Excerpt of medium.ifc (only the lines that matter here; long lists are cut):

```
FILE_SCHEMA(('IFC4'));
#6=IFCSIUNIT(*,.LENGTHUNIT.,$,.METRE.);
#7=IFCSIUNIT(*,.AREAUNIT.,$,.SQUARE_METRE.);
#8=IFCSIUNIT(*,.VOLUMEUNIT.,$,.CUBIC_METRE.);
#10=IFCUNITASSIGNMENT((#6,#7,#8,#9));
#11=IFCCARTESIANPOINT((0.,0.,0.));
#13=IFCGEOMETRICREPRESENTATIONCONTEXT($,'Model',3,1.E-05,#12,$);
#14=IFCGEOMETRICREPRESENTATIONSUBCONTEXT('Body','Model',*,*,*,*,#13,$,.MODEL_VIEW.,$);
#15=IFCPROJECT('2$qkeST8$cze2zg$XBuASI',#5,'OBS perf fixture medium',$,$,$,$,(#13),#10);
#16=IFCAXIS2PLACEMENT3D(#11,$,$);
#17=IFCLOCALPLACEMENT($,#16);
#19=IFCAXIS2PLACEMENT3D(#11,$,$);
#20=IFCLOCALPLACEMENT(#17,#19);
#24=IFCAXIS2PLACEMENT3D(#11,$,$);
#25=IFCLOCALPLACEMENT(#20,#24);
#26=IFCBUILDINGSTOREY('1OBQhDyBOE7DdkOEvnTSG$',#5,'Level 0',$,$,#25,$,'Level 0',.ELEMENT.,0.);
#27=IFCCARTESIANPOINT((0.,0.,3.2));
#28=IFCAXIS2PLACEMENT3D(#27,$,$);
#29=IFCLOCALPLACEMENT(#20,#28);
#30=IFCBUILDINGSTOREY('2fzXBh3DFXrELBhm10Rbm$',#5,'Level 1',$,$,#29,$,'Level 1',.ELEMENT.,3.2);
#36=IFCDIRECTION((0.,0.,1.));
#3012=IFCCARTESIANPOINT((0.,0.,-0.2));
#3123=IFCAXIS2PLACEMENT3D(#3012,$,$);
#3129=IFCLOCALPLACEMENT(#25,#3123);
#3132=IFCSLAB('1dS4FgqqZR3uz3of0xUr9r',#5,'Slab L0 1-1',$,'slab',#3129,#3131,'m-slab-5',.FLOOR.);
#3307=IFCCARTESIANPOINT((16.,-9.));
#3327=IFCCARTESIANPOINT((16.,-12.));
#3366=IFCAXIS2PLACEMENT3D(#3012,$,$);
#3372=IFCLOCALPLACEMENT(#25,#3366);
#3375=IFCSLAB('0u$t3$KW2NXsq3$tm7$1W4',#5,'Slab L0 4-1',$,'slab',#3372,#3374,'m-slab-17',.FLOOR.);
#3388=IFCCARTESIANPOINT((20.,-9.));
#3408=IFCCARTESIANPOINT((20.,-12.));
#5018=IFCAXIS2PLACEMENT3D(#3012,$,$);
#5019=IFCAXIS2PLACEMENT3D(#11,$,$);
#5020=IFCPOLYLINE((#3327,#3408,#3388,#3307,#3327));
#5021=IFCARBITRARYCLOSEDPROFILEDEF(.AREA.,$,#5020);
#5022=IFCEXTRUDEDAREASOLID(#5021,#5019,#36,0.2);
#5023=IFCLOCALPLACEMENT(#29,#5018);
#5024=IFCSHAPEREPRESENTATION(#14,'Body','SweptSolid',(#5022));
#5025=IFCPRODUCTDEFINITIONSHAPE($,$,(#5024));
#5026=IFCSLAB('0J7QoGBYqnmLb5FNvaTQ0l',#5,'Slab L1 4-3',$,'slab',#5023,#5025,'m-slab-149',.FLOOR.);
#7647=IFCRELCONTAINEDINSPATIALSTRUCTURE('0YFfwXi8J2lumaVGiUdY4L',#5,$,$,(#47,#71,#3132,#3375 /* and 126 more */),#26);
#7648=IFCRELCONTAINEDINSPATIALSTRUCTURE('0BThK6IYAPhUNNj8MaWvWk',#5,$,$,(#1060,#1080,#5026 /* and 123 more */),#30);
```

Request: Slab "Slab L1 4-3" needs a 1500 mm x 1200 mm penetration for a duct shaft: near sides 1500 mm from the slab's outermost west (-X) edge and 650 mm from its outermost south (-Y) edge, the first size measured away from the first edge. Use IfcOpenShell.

```python
import numpy as np
import ifcopenshell
import ifcopenshell.api.feature
import ifcopenshell.api.geometry
import ifcopenshell.api.root
import ifcopenshell.geom
import ifcopenshell.util.placement
import ifcopenshell.util.representation
import ifcopenshell.util.shape
import ifcopenshell.util.unit

model = ifcopenshell.open("medium.ifc")
unit_scale = ifcopenshell.util.unit.calculate_unit_scale(model)
settings = ifcopenshell.geom.settings()


def volume(element):
    """Net volume in cubic metres, openings subtracted."""
    shape = ifcopenshell.geom.create_shape(settings, element)
    return ifcopenshell.util.shape.get_volume(shape.geometry)


slab = model.by_id(5026)
before = volume(slab)

# Extent in the slab's own axes, in metres. The edges named are its -X and -Y sides.
slab_shape = ifcopenshell.geom.create_shape(settings, slab)
vertices = ifcopenshell.util.shape.get_vertices(slab_shape.geometry)
x_min, y_min, bottom = vertices.min(axis=0)
top = vertices[:, 2].max()

opening = ifcopenshell.api.root.create_entity(model, ifc_class="IfcOpeningElement", name="Duct shaft opening", predefined_type="OPENING")
context = ifcopenshell.util.representation.get_context(model, "Model", "Body", "MODEL_VIEW")
width, depth = 1.5, 1.2
outline = [(0.0, 0.0), (width, 0.0), (width, depth), (0.0, depth), (0.0, 0.0)]
# Overshoot both faces by 50 mm so the cut is clean.
shape = ifcopenshell.api.geometry.add_slab_representation(
    model, context=context, depth=top - bottom + 0.1, polyline=outline
)
ifcopenshell.api.geometry.assign_representation(model, product=opening, representation=shape)

matrix = ifcopenshell.util.placement.get_local_placement(slab.ObjectPlacement)
matrix[:, 3] = matrix @ np.append(np.array([x_min + 1.5, y_min + 0.65, bottom - 0.05]) / unit_scale, 1.0)
ifcopenshell.api.geometry.edit_object_placement(model, product=opening, matrix=matrix, is_si=False)
ifcopenshell.api.feature.add_feature(model, feature=opening, element=slab)

after = volume(slab)

print(f"slab volume {before:.3f} -> {after:.3f} m3")

model.write("medium_updated.ifc")
```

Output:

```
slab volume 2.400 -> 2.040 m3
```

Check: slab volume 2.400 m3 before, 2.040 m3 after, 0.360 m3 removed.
